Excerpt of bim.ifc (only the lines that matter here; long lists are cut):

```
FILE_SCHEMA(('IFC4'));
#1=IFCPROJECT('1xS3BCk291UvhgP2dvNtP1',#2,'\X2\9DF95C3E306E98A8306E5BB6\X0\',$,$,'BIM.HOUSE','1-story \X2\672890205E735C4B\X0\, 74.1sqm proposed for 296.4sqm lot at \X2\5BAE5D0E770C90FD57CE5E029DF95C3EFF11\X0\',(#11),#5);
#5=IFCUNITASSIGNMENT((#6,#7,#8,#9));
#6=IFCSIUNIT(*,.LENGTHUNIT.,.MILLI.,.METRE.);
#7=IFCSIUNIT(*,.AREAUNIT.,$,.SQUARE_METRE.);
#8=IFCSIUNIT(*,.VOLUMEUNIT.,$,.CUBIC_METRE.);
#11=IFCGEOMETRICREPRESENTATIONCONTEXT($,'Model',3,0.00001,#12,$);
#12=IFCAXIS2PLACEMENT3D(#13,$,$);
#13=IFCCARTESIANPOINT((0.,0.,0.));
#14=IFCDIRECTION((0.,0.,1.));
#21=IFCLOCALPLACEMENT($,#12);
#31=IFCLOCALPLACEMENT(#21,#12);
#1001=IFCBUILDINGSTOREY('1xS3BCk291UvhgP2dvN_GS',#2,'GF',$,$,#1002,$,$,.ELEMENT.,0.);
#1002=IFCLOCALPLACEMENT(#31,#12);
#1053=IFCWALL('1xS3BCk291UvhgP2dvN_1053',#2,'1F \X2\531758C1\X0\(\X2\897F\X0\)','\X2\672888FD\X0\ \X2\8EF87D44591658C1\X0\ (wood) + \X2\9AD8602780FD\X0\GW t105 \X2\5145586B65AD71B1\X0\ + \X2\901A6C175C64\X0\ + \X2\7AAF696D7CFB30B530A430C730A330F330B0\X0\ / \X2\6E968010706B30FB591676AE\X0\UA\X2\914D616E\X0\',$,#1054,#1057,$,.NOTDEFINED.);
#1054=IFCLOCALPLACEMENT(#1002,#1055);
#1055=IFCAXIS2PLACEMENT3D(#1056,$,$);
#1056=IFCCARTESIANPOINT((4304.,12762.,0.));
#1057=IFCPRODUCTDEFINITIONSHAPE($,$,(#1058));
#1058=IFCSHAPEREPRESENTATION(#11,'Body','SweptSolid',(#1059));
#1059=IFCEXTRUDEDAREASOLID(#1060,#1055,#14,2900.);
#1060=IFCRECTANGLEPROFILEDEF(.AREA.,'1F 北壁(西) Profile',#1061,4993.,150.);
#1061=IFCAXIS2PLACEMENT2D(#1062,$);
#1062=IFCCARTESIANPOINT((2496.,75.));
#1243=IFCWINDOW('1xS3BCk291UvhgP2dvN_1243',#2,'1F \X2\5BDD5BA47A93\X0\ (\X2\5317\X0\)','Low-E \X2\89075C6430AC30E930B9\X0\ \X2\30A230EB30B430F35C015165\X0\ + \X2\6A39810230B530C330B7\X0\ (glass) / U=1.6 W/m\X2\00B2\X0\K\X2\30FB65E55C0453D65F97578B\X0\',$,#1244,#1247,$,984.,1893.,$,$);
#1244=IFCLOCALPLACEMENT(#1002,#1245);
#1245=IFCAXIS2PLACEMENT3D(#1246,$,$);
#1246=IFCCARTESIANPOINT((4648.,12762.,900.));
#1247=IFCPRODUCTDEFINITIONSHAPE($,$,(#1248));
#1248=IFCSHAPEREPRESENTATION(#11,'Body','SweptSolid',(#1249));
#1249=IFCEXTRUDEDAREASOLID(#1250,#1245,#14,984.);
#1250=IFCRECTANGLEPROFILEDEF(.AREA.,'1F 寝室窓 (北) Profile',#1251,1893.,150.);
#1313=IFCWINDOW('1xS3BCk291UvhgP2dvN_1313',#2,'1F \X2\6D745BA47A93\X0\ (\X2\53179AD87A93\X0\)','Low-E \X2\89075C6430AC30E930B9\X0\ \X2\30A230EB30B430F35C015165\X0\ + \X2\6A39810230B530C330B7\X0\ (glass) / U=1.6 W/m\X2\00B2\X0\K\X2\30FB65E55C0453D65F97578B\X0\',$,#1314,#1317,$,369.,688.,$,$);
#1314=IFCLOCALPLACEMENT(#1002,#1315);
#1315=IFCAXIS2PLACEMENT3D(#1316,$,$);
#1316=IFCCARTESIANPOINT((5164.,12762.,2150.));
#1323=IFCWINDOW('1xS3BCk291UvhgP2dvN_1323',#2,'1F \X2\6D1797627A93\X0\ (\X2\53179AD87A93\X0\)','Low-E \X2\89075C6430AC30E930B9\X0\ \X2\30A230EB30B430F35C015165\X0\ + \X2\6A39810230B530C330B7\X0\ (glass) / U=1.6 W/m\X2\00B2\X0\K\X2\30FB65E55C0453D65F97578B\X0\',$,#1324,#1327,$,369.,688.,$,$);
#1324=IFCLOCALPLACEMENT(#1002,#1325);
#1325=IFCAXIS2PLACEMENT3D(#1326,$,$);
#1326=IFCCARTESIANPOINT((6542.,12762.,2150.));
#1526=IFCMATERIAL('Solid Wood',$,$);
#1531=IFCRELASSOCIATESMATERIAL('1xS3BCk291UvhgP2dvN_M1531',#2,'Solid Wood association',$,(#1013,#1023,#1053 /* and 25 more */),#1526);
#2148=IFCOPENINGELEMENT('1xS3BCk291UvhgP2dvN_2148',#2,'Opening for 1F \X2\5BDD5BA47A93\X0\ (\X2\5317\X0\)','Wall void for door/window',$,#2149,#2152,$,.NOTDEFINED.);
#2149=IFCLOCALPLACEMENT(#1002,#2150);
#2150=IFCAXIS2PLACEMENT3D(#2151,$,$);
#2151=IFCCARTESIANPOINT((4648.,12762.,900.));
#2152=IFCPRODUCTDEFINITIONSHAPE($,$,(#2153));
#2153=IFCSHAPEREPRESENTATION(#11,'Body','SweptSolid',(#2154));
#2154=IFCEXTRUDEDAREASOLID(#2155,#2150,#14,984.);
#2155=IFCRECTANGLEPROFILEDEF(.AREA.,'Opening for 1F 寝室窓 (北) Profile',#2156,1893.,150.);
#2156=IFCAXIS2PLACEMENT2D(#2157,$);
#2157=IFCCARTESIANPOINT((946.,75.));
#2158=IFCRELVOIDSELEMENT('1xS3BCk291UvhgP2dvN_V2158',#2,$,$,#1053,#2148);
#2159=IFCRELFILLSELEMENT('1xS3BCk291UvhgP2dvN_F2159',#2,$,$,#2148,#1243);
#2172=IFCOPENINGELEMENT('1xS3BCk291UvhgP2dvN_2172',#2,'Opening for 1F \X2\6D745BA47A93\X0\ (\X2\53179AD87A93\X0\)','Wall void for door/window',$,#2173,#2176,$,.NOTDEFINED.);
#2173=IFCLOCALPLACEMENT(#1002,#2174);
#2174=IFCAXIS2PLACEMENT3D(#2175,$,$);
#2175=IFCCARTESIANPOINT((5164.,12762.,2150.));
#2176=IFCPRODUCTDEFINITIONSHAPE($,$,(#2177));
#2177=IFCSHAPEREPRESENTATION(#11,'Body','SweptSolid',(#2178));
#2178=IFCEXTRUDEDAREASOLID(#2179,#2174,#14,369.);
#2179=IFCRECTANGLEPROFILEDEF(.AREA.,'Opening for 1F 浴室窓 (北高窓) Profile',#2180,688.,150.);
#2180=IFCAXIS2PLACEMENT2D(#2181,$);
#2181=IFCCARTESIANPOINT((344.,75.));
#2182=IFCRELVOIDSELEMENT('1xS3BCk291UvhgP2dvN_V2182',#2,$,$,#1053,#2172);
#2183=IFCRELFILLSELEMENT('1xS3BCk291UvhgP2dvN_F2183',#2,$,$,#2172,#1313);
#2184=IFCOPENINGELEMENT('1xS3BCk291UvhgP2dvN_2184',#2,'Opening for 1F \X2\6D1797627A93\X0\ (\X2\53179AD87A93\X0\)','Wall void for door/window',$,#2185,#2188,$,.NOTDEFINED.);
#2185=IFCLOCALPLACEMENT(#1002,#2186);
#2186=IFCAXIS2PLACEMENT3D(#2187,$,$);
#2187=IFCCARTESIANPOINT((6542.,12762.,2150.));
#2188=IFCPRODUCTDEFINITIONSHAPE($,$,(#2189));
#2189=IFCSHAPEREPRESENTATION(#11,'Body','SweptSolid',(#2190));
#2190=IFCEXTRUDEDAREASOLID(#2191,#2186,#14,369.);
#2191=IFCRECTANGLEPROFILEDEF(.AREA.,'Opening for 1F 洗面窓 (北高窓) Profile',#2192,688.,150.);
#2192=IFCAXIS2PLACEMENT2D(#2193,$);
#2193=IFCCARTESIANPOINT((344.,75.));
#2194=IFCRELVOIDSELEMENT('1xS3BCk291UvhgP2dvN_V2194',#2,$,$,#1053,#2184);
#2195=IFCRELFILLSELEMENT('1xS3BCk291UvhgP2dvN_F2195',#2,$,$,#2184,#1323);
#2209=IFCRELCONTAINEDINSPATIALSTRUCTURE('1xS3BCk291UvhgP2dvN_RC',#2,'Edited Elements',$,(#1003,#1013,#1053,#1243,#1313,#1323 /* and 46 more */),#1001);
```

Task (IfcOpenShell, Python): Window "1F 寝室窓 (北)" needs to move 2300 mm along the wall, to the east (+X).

```python
import ifcopenshell
import ifcopenshell.api.geometry
import ifcopenshell.util.placement

model = ifcopenshell.open("bim.ifc")

window = model.by_id(1243)
opening = window.FillsVoids[0].RelatingOpeningElement
wall = opening.VoidsElements[0].RelatingBuildingElement

wall_matrix = ifcopenshell.util.placement.get_local_placement(wall.ObjectPlacement)
shift = wall_matrix[:3, 0] * 2300.0
before = ifcopenshell.util.placement.get_local_placement(window.ObjectPlacement)[:3, 3].copy()

# The window is not placed relative to its opening, so move both.
for product in (opening, window):
    matrix = ifcopenshell.util.placement.get_local_placement(product.ObjectPlacement)
    matrix[:3, 3] += shift
    ifcopenshell.api.geometry.edit_object_placement(model, product=product, matrix=matrix, is_si=False)

after = ifcopenshell.util.placement.get_local_placement(window.ObjectPlacement)[:3, 3]
print("window moved by", (after - before).round(3) + 0.0)

model.write("bim_rev.ifc")
```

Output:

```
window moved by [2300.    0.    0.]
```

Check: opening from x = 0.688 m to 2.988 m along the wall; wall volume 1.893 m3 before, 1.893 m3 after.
